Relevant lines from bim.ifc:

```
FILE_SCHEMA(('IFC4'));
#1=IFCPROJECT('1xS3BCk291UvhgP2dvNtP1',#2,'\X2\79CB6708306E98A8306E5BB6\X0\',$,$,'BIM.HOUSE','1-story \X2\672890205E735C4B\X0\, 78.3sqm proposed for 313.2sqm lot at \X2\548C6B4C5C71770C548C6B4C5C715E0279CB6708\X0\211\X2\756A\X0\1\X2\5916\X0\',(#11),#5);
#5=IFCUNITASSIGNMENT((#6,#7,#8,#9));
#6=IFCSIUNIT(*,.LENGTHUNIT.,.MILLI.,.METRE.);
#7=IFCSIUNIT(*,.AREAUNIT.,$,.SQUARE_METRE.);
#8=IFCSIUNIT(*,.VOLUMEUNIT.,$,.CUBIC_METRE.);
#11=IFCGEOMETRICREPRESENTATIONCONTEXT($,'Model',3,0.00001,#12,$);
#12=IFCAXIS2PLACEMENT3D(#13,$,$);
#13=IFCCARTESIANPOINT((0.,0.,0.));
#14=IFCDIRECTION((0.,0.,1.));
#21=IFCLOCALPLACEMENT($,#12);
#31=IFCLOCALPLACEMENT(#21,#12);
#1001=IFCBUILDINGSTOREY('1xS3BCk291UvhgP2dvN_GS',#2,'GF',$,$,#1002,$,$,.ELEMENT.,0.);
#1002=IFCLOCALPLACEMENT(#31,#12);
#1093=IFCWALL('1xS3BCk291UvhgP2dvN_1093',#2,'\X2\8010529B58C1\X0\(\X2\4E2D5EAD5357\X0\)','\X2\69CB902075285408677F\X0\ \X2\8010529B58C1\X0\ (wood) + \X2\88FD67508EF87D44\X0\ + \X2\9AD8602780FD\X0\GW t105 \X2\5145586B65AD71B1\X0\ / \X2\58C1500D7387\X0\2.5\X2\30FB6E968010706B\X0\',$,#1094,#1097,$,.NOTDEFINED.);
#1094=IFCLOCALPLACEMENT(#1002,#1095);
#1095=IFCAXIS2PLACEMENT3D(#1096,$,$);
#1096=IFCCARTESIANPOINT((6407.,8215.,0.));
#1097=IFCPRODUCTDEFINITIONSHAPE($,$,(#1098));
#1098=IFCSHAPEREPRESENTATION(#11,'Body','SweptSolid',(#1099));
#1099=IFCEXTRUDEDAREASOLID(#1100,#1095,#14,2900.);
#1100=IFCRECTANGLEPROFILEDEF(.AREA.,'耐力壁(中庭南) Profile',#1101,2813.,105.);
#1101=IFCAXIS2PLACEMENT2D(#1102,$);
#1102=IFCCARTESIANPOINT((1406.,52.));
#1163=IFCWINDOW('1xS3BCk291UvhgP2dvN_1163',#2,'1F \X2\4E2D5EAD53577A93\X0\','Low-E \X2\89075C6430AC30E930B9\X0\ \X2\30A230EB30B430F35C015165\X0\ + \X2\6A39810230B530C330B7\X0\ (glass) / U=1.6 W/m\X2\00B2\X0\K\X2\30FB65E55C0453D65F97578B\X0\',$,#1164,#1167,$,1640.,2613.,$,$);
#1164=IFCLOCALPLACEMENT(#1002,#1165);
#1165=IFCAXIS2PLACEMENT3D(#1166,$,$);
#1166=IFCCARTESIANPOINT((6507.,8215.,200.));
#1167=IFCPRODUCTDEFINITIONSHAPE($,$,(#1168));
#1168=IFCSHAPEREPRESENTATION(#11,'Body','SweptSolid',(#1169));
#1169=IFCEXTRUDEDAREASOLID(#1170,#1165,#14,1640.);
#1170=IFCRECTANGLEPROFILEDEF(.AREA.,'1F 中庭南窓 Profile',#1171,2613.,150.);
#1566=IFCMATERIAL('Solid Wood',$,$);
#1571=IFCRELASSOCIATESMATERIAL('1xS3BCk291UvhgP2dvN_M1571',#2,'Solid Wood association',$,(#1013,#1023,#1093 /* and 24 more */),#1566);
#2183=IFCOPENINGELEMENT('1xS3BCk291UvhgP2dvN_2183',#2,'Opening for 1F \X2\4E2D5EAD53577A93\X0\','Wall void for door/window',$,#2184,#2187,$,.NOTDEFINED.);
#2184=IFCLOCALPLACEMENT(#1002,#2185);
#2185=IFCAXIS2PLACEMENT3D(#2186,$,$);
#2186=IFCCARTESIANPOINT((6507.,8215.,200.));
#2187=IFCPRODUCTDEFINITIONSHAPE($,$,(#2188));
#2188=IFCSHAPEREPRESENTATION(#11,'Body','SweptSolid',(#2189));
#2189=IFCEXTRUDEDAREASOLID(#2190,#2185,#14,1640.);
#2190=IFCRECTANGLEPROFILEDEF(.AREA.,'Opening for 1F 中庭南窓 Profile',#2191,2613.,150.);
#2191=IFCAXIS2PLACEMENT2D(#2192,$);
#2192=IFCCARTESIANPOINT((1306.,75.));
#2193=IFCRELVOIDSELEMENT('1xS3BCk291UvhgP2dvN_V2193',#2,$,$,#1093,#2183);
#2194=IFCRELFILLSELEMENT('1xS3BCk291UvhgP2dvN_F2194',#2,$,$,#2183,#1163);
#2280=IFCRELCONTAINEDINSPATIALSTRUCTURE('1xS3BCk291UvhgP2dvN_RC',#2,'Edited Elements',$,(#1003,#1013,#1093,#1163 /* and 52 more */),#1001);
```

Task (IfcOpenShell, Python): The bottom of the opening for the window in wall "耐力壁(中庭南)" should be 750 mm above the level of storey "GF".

```python
import numpy as np
import ifcopenshell
import ifcopenshell.api.geometry
import ifcopenshell.geom
import ifcopenshell.util.element
import ifcopenshell.util.placement
import ifcopenshell.util.shape
import ifcopenshell.util.unit

model = ifcopenshell.open("bim.ifc")
unit_scale = ifcopenshell.util.unit.calculate_unit_scale(model)

window = model.by_id(1163)
opening = window.FillsVoids[0].RelatingOpeningElement
storey = ifcopenshell.util.element.get_container(window, ifc_class="IfcBuildingStorey")
level = ifcopenshell.util.placement.get_local_placement(storey.ObjectPlacement)[2, 3]

# The opening's origin need not be at the sill, so measure its lowest point.
shape = ifcopenshell.geom.create_shape(ifcopenshell.geom.settings(), opening)
bottom = ifcopenshell.util.shape.get_shape_bottom_elevation(shape, shape.geometry) / unit_scale
dz = level + 0.75 / unit_scale - bottom

shift = np.array([0.0, 0.0, dz])
# The window is not placed relative to its opening, so move both.
for product in (opening, window):
    matrix = ifcopenshell.util.placement.get_local_placement(product.ObjectPlacement)
    matrix[:3, 3] += shift
    ifcopenshell.api.geometry.edit_object_placement(model, product=product, matrix=matrix, is_si=False)

print(f"moved by {dz * unit_scale:+.3f} m")

model.write("bim_updated.ifc")
```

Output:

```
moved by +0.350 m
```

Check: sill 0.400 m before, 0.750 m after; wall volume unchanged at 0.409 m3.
